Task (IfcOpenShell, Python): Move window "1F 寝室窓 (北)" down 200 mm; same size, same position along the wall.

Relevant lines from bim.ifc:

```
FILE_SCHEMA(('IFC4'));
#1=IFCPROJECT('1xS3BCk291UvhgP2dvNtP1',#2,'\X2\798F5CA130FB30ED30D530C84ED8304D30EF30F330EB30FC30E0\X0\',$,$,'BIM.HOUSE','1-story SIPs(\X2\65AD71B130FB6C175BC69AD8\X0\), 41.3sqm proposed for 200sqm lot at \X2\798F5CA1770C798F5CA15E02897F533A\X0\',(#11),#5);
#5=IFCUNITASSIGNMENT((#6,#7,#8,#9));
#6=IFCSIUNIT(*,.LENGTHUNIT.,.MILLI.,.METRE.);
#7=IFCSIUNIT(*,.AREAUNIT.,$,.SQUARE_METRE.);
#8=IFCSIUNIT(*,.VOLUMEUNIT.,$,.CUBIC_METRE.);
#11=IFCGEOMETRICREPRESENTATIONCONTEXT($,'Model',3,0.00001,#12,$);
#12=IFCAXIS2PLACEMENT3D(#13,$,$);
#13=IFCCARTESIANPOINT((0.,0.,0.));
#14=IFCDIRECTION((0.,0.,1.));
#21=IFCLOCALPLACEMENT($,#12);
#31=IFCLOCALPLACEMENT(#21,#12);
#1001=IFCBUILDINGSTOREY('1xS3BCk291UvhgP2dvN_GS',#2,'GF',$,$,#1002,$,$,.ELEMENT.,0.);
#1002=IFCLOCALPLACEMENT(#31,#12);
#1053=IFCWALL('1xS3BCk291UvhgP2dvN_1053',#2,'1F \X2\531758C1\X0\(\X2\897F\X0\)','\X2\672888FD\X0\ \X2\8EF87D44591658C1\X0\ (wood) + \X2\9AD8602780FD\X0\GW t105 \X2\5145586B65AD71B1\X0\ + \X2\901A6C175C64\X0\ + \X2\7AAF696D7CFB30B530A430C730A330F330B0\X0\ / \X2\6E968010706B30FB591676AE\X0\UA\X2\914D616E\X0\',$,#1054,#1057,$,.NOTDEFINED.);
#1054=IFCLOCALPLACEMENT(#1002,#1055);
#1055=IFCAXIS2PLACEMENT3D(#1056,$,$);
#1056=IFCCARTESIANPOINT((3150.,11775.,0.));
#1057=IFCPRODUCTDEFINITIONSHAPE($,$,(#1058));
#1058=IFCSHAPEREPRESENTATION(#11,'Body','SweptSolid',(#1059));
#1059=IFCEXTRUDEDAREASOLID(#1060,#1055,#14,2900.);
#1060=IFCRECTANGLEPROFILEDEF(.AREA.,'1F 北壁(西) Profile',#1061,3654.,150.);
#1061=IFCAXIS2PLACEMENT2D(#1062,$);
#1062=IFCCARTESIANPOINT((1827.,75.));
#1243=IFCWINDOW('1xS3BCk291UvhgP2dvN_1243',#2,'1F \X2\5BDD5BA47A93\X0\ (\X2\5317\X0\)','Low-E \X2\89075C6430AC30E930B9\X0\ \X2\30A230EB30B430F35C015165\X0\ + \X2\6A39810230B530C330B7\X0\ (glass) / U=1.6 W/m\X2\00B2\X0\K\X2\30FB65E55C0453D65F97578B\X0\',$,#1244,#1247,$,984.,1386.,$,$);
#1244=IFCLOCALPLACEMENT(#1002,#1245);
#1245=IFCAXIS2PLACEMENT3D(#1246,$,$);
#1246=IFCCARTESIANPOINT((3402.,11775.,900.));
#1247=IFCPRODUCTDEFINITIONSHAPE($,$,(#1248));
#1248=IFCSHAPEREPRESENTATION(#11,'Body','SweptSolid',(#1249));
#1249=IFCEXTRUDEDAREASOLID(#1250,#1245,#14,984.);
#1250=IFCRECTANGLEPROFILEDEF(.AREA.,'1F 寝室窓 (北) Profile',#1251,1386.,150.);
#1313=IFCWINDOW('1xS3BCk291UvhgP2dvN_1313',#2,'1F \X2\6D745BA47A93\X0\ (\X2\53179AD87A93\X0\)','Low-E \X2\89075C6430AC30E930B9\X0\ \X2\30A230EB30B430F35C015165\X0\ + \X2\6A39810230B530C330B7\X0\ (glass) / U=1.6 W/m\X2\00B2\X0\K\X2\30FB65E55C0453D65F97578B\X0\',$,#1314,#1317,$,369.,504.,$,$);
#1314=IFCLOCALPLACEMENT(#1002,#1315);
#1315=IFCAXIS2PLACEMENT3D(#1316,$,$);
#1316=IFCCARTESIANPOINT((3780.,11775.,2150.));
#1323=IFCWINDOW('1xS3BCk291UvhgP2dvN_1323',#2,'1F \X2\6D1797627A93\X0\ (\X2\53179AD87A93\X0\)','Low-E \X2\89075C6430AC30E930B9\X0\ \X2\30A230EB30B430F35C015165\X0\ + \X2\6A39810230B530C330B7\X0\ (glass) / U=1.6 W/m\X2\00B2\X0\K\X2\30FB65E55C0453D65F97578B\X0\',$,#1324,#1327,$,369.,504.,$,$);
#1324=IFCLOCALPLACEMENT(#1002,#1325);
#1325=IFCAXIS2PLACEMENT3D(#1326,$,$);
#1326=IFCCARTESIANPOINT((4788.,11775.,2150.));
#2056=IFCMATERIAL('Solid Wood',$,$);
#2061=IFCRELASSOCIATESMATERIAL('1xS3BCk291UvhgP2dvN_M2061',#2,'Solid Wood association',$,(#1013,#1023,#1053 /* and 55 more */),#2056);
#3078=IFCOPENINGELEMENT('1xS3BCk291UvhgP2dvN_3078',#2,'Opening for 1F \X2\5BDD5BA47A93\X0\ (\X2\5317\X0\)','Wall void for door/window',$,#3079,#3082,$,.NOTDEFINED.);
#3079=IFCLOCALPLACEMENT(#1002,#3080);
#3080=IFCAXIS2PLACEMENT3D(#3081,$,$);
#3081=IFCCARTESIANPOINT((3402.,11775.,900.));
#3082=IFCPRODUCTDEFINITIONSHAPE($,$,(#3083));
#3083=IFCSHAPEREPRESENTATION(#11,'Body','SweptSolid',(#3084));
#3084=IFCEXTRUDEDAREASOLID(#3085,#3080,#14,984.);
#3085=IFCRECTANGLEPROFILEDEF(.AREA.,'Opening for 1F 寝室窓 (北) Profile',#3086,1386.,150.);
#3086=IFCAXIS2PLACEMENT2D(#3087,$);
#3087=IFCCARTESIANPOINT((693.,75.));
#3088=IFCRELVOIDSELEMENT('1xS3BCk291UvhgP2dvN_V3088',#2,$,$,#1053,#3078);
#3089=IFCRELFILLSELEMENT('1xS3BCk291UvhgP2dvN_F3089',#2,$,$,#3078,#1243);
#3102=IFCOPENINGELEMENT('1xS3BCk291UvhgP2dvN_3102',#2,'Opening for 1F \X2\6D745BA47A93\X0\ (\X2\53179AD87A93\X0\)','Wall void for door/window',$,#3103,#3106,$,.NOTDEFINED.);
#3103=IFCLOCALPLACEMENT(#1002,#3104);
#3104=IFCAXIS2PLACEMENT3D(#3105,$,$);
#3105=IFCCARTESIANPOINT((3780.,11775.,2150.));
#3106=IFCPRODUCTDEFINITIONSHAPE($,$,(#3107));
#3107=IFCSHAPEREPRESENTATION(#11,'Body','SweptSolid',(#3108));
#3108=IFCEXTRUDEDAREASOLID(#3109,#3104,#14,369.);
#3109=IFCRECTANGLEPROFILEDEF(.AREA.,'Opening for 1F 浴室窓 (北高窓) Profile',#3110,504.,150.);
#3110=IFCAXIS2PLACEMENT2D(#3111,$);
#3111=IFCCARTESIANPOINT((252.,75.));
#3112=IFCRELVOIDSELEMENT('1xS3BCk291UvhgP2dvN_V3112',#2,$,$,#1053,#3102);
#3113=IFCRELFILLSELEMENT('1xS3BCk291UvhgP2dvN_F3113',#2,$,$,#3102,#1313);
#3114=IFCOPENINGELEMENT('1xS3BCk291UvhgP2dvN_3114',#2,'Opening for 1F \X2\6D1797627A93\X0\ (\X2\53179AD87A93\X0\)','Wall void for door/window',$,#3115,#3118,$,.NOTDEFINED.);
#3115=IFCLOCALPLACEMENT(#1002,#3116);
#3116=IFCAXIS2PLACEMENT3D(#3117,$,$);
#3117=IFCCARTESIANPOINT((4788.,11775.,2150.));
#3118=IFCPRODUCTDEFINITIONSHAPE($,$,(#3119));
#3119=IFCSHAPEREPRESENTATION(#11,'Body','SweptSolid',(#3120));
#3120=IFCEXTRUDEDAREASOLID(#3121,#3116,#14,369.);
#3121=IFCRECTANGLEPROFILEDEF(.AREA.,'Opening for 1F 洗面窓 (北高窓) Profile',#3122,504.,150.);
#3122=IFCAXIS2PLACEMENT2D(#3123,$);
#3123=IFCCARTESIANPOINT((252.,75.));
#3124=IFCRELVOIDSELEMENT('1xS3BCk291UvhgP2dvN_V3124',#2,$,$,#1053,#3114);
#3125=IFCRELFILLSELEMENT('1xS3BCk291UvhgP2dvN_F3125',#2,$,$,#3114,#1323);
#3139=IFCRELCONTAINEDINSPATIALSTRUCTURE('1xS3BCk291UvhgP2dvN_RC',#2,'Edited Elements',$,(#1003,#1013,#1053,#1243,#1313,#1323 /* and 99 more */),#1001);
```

```python
import numpy as np
import ifcopenshell
import ifcopenshell.api.geometry
import ifcopenshell.util.placement
import ifcopenshell.util.unit

model = ifcopenshell.open("bim.ifc")
unit_scale = ifcopenshell.util.unit.calculate_unit_scale(model)

window = model.by_guid("1xS3BCk291UvhgP2dvN_1243")
opening = window.FillsVoids[0].RelatingOpeningElement
dz = -0.2 / unit_scale

shift = np.array([0.0, 0.0, dz])
# The window is not placed relative to its opening, so move both.
for product in (opening, window):
    matrix = ifcopenshell.util.placement.get_local_placement(product.ObjectPlacement)
    matrix[:3, 3] += shift
    ifcopenshell.api.geometry.edit_object_placement(model, product=product, matrix=matrix, is_si=False)

print(f"moved by {dz * unit_scale:+.3f} m")

model.write("bim_updated.ifc")
```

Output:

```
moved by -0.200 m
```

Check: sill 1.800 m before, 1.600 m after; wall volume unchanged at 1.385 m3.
